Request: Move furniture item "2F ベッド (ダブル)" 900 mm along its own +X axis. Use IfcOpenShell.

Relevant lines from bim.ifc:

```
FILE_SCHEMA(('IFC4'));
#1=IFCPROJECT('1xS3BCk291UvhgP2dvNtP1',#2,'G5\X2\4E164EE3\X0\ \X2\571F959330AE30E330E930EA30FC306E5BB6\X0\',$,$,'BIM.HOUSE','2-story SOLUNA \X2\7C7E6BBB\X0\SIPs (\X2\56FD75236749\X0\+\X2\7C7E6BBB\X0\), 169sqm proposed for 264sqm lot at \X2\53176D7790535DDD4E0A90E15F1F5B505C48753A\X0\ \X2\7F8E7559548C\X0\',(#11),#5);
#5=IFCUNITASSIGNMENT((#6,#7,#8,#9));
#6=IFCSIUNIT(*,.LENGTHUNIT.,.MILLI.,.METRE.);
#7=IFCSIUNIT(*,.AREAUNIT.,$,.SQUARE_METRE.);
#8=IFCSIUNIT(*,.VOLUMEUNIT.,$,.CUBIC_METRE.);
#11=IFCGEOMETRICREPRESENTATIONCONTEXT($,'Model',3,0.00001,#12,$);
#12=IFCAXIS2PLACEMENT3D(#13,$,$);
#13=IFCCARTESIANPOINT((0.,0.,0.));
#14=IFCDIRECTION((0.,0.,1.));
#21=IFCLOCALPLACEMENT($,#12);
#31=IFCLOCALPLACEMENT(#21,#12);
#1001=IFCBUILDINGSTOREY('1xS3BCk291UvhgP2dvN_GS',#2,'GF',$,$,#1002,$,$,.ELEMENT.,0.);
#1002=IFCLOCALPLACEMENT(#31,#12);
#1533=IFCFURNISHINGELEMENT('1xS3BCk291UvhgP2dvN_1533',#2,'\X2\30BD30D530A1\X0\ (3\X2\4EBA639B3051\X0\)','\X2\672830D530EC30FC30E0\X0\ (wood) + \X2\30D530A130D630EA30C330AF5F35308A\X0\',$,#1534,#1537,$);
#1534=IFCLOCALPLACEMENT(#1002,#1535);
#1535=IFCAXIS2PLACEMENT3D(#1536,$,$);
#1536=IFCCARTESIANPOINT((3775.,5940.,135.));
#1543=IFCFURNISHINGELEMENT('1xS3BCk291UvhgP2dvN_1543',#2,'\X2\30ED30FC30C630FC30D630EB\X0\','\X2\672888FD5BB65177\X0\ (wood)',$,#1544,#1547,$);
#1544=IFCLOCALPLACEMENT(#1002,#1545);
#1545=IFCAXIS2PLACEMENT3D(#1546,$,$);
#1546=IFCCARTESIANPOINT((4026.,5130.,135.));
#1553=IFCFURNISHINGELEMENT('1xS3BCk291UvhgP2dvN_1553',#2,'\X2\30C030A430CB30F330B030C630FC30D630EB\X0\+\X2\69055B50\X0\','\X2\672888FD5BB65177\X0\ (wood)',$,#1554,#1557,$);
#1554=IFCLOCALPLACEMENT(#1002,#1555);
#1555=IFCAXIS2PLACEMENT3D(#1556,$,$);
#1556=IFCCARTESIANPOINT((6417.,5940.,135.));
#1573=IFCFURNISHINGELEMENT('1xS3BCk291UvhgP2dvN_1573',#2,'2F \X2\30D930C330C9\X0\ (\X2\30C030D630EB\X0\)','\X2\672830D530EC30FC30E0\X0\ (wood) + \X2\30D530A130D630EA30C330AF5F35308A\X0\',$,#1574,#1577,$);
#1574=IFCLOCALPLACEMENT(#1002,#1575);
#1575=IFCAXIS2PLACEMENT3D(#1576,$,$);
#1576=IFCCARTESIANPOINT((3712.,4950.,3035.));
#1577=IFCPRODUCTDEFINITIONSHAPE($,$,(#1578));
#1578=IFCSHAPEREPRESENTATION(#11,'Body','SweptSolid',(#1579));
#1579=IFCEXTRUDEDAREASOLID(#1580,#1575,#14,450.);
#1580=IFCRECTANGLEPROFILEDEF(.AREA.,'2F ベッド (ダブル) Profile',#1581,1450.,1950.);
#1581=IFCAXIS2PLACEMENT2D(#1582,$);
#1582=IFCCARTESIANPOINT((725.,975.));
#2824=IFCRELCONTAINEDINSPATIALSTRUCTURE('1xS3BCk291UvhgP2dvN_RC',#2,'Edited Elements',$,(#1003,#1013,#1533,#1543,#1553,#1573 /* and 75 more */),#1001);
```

```python
import ifcopenshell
import ifcopenshell.api.geometry
import ifcopenshell.util.placement
import ifcopenshell.util.unit

model = ifcopenshell.open("bim.ifc")
unit_scale = ifcopenshell.util.unit.calculate_unit_scale(model)

item = model.by_guid("1xS3BCk291UvhgP2dvN_1573")
matrix = ifcopenshell.util.placement.get_local_placement(item.ObjectPlacement)
matrix[:3, 3] += matrix[:3, 0] * 0.9 / unit_scale
ifcopenshell.api.geometry.edit_object_placement(model, product=item, matrix=matrix, is_si=False)

print(ifcopenshell.util.placement.get_local_placement(item.ObjectPlacement).round(3) + 0.0)

model.write("bim_rev.ifc")
```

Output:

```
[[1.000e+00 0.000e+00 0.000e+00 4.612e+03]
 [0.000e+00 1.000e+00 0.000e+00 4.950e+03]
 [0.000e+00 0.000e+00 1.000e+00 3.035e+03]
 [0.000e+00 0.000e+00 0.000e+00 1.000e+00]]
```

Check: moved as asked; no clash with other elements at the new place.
